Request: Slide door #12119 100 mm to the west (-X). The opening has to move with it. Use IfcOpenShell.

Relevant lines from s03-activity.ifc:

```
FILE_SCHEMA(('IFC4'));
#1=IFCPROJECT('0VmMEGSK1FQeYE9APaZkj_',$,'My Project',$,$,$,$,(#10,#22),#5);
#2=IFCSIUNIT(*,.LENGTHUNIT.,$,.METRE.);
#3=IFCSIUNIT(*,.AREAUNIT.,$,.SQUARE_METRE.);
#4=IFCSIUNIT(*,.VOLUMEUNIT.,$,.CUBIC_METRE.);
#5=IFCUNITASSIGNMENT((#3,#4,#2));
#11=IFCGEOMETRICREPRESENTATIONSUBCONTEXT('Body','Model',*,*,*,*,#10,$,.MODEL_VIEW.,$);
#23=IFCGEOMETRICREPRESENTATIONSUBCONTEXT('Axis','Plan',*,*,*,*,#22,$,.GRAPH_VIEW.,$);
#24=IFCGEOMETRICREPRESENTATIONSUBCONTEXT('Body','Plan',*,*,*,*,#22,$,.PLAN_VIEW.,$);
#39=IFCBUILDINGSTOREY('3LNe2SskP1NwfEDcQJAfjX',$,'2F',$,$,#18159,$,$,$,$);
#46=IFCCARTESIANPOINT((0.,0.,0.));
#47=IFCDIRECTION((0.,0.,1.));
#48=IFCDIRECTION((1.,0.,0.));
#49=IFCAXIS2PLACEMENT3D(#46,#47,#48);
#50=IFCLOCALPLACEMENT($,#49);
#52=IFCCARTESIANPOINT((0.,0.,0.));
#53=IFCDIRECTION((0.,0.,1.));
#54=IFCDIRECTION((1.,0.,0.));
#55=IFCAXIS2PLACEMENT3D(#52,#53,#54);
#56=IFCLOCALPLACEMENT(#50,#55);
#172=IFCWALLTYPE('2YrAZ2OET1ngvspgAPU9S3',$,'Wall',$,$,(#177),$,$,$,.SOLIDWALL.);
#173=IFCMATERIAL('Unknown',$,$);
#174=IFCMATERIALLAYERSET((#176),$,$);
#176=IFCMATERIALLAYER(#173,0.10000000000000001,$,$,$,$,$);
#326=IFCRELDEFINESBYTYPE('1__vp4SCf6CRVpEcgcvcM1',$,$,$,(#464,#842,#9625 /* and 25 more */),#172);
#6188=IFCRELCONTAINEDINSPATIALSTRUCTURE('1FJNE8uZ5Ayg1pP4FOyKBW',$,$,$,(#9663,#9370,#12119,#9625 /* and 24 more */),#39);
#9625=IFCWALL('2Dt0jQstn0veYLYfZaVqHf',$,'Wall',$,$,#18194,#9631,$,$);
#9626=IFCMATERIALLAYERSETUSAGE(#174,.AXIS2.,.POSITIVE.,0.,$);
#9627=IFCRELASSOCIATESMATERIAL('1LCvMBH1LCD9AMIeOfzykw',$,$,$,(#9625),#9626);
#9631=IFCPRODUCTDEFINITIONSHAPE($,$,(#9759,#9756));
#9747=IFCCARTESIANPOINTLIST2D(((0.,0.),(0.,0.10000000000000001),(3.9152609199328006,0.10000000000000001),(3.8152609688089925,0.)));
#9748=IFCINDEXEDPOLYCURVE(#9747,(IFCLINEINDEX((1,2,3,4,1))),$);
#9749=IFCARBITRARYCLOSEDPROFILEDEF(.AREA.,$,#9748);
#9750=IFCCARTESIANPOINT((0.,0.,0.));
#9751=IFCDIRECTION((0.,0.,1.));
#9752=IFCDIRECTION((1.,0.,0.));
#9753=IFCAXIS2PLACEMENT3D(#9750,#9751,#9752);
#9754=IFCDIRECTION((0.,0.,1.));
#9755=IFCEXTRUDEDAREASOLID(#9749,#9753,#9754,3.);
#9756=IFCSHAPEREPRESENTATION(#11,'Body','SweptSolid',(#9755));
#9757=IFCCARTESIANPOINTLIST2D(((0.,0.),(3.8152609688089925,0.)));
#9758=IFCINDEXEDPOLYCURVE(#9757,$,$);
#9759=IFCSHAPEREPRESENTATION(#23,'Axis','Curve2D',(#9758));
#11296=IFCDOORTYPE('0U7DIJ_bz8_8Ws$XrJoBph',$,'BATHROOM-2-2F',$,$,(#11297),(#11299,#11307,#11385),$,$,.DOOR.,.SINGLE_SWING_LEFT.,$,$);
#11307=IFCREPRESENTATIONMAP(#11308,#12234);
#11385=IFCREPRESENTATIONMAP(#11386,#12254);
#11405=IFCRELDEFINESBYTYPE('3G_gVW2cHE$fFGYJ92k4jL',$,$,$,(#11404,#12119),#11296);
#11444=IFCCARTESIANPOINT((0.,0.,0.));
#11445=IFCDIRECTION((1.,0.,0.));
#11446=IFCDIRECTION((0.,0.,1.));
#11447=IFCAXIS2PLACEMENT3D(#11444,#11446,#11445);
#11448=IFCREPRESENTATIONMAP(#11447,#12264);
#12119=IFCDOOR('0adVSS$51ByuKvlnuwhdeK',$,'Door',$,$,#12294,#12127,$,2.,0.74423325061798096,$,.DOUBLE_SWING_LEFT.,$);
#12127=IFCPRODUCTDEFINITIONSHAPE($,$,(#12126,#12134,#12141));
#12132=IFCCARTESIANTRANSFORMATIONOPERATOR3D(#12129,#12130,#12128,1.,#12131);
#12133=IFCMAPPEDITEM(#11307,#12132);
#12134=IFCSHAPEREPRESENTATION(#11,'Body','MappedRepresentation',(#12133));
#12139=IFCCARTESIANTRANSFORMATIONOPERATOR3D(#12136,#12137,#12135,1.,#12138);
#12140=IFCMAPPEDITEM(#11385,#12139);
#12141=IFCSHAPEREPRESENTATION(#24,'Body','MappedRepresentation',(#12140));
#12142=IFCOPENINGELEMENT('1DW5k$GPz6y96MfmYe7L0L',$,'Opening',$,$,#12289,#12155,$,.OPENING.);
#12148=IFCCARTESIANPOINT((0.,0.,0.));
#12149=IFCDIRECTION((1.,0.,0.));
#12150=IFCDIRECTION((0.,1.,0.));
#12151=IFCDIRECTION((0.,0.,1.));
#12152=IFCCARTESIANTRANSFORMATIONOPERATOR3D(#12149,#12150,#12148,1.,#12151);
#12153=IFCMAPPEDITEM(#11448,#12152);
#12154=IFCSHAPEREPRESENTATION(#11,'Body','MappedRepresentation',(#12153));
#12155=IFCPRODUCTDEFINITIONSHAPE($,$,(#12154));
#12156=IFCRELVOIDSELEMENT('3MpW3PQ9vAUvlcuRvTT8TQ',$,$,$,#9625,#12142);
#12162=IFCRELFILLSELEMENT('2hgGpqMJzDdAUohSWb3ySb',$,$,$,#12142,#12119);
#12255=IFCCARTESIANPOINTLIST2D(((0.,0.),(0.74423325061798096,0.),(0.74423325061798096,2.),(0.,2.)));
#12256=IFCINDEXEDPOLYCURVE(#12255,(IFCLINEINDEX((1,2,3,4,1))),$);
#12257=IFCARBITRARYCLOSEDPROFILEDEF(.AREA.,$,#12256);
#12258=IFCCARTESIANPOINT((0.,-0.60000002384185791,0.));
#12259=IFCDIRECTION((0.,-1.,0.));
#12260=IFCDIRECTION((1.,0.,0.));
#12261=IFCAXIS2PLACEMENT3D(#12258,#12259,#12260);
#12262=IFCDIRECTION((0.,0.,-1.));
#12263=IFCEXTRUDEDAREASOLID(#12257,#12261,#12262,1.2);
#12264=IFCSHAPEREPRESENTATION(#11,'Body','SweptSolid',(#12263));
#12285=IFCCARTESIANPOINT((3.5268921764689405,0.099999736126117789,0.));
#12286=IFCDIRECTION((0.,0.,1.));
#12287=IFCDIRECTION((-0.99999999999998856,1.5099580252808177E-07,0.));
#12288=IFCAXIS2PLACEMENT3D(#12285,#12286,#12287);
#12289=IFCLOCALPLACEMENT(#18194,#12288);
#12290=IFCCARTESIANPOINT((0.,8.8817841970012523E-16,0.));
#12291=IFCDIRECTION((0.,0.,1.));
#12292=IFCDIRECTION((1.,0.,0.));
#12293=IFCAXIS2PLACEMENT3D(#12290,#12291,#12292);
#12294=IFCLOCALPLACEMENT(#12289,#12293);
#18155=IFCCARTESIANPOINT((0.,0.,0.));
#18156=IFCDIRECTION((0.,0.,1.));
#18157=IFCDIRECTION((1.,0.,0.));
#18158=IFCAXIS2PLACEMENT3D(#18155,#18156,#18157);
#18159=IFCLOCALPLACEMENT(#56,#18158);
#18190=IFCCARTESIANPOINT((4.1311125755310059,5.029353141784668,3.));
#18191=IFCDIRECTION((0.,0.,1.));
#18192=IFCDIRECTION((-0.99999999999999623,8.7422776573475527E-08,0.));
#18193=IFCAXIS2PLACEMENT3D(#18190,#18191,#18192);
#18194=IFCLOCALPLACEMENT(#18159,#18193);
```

```python
import ifcopenshell
import ifcopenshell.api.geometry
import ifcopenshell.util.placement
import ifcopenshell.util.unit

model = ifcopenshell.open("s03-activity.ifc")
unit_scale = ifcopenshell.util.unit.calculate_unit_scale(model)

door = model.by_id(12119)
opening = door.FillsVoids[0].RelatingOpeningElement
wall = opening.VoidsElements[0].RelatingBuildingElement

wall_matrix = ifcopenshell.util.placement.get_local_placement(wall.ObjectPlacement)
shift = wall_matrix[:3, 0] * 0.1 / unit_scale
before = ifcopenshell.util.placement.get_local_placement(door.ObjectPlacement)[:3, 3].copy()

# The door is placed relative to its opening, so it follows when the opening moves.
matrix = ifcopenshell.util.placement.get_local_placement(opening.ObjectPlacement)
matrix[:3, 3] += shift
ifcopenshell.api.geometry.edit_object_placement(
    model, product=opening, matrix=matrix, is_si=False, should_transform_children=True
)

after = ifcopenshell.util.placement.get_local_placement(door.ObjectPlacement)[:3, 3]
print("door moved by", (after - before).round(3) + 0.0)

model.write("s03-activity_updated.ifc")
```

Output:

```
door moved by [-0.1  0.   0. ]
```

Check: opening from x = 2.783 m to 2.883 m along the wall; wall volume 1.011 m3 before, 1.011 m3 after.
